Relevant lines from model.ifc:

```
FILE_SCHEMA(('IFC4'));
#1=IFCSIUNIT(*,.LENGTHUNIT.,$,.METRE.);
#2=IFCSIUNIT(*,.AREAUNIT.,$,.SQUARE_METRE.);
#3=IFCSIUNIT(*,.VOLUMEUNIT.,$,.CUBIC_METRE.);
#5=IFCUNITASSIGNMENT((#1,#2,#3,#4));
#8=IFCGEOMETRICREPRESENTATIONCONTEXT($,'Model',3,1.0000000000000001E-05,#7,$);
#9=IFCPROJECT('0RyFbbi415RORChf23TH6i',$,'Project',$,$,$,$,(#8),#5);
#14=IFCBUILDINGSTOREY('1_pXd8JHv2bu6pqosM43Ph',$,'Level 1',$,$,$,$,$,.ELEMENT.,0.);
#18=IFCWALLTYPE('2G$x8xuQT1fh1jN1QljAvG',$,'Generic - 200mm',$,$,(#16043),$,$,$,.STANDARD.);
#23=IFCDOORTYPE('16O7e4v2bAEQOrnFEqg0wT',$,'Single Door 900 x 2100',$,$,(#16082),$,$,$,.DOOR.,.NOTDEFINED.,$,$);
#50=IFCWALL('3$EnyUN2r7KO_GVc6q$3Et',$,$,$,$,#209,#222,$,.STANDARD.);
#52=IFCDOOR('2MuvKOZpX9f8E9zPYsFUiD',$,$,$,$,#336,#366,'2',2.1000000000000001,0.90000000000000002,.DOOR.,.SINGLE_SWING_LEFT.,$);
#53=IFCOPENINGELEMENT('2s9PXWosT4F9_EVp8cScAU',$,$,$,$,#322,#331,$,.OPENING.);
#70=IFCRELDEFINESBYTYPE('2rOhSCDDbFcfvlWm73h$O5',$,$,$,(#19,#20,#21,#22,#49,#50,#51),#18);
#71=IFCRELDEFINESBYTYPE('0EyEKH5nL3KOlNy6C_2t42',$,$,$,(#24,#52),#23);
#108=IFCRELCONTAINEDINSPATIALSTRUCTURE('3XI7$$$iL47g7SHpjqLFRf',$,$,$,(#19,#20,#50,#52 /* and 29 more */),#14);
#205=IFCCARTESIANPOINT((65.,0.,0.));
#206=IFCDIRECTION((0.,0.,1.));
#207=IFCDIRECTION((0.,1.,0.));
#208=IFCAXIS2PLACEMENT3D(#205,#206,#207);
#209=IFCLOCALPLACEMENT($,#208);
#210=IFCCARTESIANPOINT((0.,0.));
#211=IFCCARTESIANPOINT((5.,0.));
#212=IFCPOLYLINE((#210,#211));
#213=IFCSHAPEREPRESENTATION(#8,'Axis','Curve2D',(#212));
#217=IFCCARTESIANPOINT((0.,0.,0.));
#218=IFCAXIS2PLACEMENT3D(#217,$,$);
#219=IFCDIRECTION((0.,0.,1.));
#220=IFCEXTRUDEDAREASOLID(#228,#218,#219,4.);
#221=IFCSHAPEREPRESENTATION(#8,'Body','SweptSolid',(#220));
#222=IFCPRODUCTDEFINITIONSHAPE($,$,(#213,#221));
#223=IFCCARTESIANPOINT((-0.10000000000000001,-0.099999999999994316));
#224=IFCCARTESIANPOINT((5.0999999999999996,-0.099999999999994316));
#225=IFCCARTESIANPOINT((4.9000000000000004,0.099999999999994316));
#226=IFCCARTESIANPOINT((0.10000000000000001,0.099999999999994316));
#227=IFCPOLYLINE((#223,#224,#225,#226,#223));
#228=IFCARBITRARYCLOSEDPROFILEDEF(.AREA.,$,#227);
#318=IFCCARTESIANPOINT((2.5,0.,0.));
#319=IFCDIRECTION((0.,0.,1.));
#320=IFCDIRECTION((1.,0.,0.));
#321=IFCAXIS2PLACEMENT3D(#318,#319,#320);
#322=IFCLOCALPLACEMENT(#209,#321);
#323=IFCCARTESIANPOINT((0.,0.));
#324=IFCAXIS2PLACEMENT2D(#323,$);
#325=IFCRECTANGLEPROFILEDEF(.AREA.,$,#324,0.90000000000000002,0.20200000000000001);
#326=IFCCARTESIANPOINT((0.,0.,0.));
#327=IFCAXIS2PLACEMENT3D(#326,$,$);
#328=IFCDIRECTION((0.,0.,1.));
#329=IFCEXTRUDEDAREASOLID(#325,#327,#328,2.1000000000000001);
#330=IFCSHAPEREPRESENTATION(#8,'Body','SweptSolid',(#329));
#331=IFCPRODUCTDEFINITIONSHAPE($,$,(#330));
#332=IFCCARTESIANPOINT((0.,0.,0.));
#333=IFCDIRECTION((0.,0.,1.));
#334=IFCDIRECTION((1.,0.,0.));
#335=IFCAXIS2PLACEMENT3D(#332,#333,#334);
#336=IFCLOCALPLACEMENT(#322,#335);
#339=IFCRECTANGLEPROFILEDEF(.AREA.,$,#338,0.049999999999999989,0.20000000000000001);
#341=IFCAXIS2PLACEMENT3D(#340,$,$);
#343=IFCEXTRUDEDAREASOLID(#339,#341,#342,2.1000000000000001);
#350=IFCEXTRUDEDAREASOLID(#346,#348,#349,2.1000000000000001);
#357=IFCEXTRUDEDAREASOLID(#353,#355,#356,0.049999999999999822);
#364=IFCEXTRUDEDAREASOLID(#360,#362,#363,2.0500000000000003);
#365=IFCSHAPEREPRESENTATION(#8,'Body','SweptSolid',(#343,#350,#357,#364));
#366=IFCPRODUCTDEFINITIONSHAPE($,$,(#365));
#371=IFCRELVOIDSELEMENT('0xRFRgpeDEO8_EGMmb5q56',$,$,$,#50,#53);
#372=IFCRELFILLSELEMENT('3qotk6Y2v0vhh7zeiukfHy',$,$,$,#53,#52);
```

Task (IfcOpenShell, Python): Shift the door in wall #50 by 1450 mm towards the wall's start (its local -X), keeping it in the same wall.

```python
import ifcopenshell
import ifcopenshell.api.geometry
import ifcopenshell.util.placement
import ifcopenshell.util.unit

model = ifcopenshell.open("model.ifc")
unit_scale = ifcopenshell.util.unit.calculate_unit_scale(model)

door = model.by_id(52)
opening = door.FillsVoids[0].RelatingOpeningElement
wall = opening.VoidsElements[0].RelatingBuildingElement

wall_matrix = ifcopenshell.util.placement.get_local_placement(wall.ObjectPlacement)
shift = wall_matrix[:3, 0] * -1.45 / unit_scale
before = ifcopenshell.util.placement.get_local_placement(door.ObjectPlacement)[:3, 3].copy()

# The door is placed relative to its opening, so it follows when the opening moves.
matrix = ifcopenshell.util.placement.get_local_placement(opening.ObjectPlacement)
matrix[:3, 3] += shift
ifcopenshell.api.geometry.edit_object_placement(
    model, product=opening, matrix=matrix, is_si=False, should_transform_children=True
)

after = ifcopenshell.util.placement.get_local_placement(door.ObjectPlacement)[:3, 3]
print("door moved by", (after - before).round(3) + 0.0)

model.write("model_updated.ifc")
```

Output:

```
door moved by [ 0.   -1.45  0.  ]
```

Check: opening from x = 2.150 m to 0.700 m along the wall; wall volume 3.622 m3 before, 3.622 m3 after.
